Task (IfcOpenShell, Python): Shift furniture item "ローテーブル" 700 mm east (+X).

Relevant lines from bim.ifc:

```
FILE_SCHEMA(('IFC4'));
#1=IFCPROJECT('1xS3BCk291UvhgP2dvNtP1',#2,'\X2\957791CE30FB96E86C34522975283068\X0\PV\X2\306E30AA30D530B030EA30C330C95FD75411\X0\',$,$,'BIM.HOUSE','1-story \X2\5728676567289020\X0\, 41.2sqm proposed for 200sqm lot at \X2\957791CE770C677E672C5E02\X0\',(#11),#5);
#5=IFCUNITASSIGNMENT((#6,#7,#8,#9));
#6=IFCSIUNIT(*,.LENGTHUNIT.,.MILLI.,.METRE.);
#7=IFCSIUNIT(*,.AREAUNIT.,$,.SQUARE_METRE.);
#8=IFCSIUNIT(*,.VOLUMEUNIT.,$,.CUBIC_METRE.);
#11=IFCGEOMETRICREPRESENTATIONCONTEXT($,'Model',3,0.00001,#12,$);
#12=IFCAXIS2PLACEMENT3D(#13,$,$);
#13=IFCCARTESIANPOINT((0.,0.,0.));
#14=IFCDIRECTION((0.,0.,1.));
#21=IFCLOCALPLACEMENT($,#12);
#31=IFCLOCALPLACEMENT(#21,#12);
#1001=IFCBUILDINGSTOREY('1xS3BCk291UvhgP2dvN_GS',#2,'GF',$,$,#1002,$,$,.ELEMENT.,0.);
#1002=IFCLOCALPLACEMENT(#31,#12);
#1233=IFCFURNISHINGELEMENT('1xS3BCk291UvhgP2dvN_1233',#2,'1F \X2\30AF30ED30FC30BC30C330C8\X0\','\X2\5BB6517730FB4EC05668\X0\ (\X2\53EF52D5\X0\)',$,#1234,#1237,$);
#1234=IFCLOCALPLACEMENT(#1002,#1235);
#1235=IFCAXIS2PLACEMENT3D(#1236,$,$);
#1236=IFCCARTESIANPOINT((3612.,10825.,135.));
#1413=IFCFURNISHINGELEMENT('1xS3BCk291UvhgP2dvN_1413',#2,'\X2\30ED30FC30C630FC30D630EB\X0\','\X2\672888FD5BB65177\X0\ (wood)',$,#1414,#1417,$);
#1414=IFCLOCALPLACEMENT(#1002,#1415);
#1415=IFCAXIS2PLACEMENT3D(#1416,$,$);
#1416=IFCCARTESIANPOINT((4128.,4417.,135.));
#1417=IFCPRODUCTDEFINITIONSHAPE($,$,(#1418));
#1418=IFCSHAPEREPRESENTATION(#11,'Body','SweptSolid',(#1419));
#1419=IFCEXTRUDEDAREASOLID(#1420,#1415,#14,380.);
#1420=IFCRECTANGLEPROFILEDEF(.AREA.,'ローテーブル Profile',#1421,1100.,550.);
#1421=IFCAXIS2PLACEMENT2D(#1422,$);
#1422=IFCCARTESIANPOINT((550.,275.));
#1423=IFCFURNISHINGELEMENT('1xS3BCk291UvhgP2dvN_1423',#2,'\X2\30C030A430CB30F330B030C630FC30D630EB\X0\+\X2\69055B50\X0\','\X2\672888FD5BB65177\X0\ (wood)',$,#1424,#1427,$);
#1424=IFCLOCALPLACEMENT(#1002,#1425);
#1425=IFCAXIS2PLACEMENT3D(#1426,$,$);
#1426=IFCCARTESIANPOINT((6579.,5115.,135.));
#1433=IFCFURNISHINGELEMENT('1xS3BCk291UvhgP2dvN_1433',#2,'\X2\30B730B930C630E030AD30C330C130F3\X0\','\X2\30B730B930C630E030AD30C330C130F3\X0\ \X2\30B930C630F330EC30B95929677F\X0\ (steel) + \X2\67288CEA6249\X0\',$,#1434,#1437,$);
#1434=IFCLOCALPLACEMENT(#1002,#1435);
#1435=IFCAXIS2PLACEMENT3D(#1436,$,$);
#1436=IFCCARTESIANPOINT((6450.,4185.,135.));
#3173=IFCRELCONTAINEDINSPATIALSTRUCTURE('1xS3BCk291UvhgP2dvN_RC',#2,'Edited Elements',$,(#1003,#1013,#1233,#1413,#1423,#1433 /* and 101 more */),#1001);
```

```python
import ifcopenshell
import ifcopenshell.api.geometry
import ifcopenshell.util.placement
import ifcopenshell.util.unit

model = ifcopenshell.open("bim.ifc")
unit_scale = ifcopenshell.util.unit.calculate_unit_scale(model)

item = model.by_id(1413)
matrix = ifcopenshell.util.placement.get_local_placement(item.ObjectPlacement)
matrix[0, 3] += 0.7 / unit_scale
ifcopenshell.api.geometry.edit_object_placement(model, product=item, matrix=matrix, is_si=False)

print(ifcopenshell.util.placement.get_local_placement(item.ObjectPlacement).round(3) + 0.0)

model.write("bim_rev.ifc")
```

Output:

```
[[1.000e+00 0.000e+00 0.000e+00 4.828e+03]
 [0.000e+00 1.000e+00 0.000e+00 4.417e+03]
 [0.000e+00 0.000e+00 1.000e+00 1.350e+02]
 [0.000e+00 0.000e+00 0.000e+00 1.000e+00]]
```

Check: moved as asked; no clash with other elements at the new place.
